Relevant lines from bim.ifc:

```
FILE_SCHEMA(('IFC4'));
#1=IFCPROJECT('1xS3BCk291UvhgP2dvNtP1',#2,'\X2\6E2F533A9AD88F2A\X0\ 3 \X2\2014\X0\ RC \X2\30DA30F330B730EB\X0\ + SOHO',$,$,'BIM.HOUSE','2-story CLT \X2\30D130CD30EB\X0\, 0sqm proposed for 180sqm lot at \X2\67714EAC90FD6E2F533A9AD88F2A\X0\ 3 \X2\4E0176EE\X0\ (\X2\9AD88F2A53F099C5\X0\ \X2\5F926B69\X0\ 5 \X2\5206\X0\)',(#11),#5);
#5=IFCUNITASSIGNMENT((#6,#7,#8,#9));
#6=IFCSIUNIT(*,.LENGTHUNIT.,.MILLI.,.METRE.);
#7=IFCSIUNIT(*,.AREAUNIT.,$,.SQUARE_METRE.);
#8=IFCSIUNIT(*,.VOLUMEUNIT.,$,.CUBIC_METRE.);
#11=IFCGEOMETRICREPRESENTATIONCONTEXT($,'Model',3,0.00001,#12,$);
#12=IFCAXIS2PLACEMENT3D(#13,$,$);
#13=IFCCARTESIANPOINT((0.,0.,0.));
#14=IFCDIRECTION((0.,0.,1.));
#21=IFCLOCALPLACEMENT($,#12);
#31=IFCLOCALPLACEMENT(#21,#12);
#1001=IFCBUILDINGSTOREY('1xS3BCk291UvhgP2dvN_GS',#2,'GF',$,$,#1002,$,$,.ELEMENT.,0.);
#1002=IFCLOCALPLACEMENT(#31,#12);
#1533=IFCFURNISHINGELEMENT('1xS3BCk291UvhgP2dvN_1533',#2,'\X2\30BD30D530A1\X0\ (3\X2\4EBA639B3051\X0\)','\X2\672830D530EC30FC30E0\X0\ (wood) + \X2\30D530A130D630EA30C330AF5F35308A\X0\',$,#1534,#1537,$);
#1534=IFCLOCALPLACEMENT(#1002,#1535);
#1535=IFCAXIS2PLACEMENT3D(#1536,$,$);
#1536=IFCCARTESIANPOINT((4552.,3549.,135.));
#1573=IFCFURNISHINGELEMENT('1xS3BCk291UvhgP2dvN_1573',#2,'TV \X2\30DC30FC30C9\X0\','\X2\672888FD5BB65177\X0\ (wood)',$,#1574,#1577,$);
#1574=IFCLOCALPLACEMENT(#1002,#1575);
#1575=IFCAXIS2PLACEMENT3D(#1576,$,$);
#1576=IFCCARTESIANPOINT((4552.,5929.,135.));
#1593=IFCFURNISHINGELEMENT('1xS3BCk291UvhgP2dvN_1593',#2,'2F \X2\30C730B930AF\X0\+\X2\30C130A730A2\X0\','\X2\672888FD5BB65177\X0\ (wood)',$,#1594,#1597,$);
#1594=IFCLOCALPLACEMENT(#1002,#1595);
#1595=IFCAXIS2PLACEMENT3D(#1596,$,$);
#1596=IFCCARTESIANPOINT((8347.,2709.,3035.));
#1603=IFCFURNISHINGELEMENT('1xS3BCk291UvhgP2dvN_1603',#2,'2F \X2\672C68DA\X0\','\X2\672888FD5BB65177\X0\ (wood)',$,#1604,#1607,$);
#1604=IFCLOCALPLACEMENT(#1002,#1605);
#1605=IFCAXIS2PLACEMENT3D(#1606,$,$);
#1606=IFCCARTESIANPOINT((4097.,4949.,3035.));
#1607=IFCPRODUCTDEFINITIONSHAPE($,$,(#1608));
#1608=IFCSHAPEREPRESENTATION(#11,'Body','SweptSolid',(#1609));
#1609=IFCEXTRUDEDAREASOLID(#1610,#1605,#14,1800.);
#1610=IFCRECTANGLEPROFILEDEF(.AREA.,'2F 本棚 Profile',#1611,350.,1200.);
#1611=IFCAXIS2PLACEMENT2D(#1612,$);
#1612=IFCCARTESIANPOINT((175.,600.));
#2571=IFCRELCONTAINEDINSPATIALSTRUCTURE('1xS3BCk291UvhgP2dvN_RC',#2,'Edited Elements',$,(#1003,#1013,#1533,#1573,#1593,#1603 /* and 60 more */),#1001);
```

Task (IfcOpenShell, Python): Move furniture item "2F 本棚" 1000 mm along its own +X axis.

```python
import ifcopenshell
import ifcopenshell.api.geometry
import ifcopenshell.util.placement

model = ifcopenshell.open("bim.ifc")

item = model.by_guid("1xS3BCk291UvhgP2dvN_1603")
matrix = ifcopenshell.util.placement.get_local_placement(item.ObjectPlacement)
matrix[:3, 3] += matrix[:3, 0] * 1000.0
ifcopenshell.api.geometry.edit_object_placement(model, product=item, matrix=matrix, is_si=False)

print(ifcopenshell.util.placement.get_local_placement(item.ObjectPlacement).round(3) + 0.0)

model.write("bim_rev.ifc")
```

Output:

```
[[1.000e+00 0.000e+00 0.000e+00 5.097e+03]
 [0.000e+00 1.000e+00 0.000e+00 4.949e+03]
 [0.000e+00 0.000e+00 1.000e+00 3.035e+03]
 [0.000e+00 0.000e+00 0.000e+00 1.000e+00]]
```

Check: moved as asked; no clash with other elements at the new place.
